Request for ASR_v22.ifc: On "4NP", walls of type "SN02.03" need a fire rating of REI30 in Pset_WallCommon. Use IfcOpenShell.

First a look at what the model holds.

```python
import ifcopenshell
import ifcopenshell.util.element

model = ifcopenshell.open("ASR_v22.ifc")
print(model.schema)
storey = next(s for s in model.by_type("IfcBuildingStorey") if s.Name == "4NP")
walls = [e for e in ifcopenshell.util.element.get_decomposition(storey) if e.is_a("IfcWall")]
seen = {}
for e in walls:
    element_type = ifcopenshell.util.element.get_type(e)
    key = (element_type.Name if element_type != e and element_type else None, ifcopenshell.util.element.get_pset(e, "Pset_WallCommon", "FireRating"))
    seen[key] = seen.get(key, 0) + 1
for (name, value), count in sorted(seen.items(), key=str):
    print(count, "x", name, "|", value)
```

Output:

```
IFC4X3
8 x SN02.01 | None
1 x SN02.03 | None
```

```python
import ifcopenshell
import ifcopenshell.api.pset
import ifcopenshell.util.element

model = ifcopenshell.open("ASR_v22.ifc")

storey = next(s for s in model.by_type("IfcBuildingStorey") if s.Name == "4NP")
walls = [e for e in ifcopenshell.util.element.get_decomposition(storey) if e.is_a("IfcWall")]

count = 0
for e in walls:
    element_type = ifcopenshell.util.element.get_type(e)
    if element_type in (None, e) or element_type.Name != "SN02.03":
        continue
    # add_pset returns the element's existing set when there is one.
    pset = ifcopenshell.api.pset.add_pset(model, product=e, name="Pset_WallCommon")
    ifcopenshell.api.pset.edit_pset(model, pset=pset, properties={"FireRating": "REI30"})
    count += 1

print(count, "walls updated")

model.write("ASR_v22_v2.ifc")
```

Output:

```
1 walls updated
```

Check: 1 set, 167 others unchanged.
